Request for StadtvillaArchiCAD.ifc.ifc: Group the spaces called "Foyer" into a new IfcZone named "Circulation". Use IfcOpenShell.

First a look at what the model holds.

```python
import ifcopenshell

model = ifcopenshell.open("StadtvillaArchiCAD.ifc.ifc")
print(model.schema)
seen = {}
for space in model.by_type("IfcSpace"):
    seen[space.LongName] = seen.get(space.LongName, 0) + 1
for name, count in sorted(seen.items(), key=str):
    print(count, "x", name)
print("zones:", [z.Name for z in model.by_type("IfcZone")][:20])
```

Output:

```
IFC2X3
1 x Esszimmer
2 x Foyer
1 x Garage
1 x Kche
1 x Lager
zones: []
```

```python
import ifcopenshell
import ifcopenshell.api.group
import ifcopenshell.api.root

model = ifcopenshell.open("StadtvillaArchiCAD.ifc.ifc")

names = {"Foyer"}
spaces = [s for s in model.by_type("IfcSpace") if s.LongName in names]

zone = ifcopenshell.api.root.create_entity(model, ifc_class="IfcZone", name="Circulation")
ifcopenshell.api.group.assign_group(model, products=spaces, group=zone)
print(len(spaces), "spaces in", zone.Name)

model.write("StadtvillaArchiCAD.ifc-out.ifc")
```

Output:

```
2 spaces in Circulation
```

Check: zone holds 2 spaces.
